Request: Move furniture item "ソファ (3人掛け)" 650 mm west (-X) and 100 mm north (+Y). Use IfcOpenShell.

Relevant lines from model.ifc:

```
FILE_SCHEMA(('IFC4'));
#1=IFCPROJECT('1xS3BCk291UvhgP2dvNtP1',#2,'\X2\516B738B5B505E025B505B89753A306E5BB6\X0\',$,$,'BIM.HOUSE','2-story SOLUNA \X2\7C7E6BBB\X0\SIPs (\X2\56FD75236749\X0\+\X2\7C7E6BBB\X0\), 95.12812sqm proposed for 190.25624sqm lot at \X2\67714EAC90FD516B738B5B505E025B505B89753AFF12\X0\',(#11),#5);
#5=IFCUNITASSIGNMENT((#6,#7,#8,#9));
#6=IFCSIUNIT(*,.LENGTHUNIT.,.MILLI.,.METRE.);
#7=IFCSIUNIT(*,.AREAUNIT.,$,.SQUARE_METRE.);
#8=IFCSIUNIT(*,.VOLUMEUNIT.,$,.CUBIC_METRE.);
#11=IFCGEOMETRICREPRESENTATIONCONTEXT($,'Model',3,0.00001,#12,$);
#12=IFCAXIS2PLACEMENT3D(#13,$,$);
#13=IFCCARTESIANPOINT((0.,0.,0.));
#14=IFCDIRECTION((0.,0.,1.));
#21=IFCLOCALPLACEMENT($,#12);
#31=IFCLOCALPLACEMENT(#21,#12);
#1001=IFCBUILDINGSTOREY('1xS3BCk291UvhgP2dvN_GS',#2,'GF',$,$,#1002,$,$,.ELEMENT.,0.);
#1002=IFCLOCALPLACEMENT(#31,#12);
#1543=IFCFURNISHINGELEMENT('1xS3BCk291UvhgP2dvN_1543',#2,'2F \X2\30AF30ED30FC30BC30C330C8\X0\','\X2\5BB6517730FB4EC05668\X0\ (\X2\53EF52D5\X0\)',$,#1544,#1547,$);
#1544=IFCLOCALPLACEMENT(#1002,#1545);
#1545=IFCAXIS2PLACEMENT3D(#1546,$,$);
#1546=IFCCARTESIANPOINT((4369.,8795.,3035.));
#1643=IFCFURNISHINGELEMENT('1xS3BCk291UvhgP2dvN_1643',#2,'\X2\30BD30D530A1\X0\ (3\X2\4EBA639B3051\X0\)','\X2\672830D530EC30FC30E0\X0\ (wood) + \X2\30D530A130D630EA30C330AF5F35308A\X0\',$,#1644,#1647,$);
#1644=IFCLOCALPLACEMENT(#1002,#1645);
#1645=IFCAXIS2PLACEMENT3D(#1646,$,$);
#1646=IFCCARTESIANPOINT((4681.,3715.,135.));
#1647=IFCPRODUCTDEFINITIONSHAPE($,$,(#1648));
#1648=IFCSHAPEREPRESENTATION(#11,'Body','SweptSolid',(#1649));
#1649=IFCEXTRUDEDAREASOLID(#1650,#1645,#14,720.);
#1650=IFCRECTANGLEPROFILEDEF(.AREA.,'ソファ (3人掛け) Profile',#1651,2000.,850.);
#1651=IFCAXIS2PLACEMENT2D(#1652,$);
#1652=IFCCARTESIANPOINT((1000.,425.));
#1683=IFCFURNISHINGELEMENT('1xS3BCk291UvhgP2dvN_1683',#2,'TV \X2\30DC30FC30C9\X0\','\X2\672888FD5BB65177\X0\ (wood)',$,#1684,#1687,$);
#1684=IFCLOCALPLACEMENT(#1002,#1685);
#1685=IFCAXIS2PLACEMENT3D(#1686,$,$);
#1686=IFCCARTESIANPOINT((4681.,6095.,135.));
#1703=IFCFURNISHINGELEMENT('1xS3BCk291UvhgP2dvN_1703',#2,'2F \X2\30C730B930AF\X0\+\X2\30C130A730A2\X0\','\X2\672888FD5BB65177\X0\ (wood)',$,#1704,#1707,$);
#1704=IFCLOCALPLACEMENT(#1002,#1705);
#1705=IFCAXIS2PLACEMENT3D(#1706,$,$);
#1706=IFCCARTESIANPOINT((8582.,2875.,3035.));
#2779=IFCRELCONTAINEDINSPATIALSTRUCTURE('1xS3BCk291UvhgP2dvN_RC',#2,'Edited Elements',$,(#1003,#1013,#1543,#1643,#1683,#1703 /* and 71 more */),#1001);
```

```python
import ifcopenshell
import ifcopenshell.api.geometry
import ifcopenshell.util.placement

model = ifcopenshell.open("model.ifc")

item = model.by_id(1643)
matrix = ifcopenshell.util.placement.get_local_placement(item.ObjectPlacement)
matrix[0, 3] -= 650.0
matrix[1, 3] += 100.0
ifcopenshell.api.geometry.edit_object_placement(model, product=item, matrix=matrix, is_si=False)

print(ifcopenshell.util.placement.get_local_placement(item.ObjectPlacement).round(3) + 0.0)

model.write("model_edited.ifc")
```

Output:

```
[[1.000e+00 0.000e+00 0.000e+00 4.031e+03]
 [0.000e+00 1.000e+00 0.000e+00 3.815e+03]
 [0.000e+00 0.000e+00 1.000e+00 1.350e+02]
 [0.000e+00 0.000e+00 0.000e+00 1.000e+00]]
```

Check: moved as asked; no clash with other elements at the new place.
